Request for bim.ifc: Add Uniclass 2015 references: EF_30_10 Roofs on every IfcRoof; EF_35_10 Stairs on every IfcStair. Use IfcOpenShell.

First a look at what the model holds.

```python
import ifcopenshell

model = ifcopenshell.open("bim.ifc")
print(model.schema)
print("classifications:", [c.Name for c in model.by_type("IfcClassification")])
for ifc_class in ("IfcDoor", "IfcRoof", "IfcStair", "IfcWall", "IfcWindow"):
    print(ifc_class, len(model.by_type(ifc_class)))
```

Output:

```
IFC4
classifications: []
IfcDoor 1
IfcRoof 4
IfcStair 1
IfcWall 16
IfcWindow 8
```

```python
import ifcopenshell
import ifcopenshell.api.classification

model = ifcopenshell.open("bim.ifc")

system = ifcopenshell.api.classification.add_classification(model, classification="Uniclass 2015")

codes = {
    "IfcRoof": ("EF_30_10", "Roofs"),
    "IfcStair": ("EF_35_10", "Stairs"),
}
for ifc_class, (code, name) in codes.items():
    products = model.by_type(ifc_class)
    ifcopenshell.api.classification.add_reference(
        model, products=products, classification=system, identification=code, name=name
    )
    print(code, len(products))

model.write("bim_edited.ifc")
```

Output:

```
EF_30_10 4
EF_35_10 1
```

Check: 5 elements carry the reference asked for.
